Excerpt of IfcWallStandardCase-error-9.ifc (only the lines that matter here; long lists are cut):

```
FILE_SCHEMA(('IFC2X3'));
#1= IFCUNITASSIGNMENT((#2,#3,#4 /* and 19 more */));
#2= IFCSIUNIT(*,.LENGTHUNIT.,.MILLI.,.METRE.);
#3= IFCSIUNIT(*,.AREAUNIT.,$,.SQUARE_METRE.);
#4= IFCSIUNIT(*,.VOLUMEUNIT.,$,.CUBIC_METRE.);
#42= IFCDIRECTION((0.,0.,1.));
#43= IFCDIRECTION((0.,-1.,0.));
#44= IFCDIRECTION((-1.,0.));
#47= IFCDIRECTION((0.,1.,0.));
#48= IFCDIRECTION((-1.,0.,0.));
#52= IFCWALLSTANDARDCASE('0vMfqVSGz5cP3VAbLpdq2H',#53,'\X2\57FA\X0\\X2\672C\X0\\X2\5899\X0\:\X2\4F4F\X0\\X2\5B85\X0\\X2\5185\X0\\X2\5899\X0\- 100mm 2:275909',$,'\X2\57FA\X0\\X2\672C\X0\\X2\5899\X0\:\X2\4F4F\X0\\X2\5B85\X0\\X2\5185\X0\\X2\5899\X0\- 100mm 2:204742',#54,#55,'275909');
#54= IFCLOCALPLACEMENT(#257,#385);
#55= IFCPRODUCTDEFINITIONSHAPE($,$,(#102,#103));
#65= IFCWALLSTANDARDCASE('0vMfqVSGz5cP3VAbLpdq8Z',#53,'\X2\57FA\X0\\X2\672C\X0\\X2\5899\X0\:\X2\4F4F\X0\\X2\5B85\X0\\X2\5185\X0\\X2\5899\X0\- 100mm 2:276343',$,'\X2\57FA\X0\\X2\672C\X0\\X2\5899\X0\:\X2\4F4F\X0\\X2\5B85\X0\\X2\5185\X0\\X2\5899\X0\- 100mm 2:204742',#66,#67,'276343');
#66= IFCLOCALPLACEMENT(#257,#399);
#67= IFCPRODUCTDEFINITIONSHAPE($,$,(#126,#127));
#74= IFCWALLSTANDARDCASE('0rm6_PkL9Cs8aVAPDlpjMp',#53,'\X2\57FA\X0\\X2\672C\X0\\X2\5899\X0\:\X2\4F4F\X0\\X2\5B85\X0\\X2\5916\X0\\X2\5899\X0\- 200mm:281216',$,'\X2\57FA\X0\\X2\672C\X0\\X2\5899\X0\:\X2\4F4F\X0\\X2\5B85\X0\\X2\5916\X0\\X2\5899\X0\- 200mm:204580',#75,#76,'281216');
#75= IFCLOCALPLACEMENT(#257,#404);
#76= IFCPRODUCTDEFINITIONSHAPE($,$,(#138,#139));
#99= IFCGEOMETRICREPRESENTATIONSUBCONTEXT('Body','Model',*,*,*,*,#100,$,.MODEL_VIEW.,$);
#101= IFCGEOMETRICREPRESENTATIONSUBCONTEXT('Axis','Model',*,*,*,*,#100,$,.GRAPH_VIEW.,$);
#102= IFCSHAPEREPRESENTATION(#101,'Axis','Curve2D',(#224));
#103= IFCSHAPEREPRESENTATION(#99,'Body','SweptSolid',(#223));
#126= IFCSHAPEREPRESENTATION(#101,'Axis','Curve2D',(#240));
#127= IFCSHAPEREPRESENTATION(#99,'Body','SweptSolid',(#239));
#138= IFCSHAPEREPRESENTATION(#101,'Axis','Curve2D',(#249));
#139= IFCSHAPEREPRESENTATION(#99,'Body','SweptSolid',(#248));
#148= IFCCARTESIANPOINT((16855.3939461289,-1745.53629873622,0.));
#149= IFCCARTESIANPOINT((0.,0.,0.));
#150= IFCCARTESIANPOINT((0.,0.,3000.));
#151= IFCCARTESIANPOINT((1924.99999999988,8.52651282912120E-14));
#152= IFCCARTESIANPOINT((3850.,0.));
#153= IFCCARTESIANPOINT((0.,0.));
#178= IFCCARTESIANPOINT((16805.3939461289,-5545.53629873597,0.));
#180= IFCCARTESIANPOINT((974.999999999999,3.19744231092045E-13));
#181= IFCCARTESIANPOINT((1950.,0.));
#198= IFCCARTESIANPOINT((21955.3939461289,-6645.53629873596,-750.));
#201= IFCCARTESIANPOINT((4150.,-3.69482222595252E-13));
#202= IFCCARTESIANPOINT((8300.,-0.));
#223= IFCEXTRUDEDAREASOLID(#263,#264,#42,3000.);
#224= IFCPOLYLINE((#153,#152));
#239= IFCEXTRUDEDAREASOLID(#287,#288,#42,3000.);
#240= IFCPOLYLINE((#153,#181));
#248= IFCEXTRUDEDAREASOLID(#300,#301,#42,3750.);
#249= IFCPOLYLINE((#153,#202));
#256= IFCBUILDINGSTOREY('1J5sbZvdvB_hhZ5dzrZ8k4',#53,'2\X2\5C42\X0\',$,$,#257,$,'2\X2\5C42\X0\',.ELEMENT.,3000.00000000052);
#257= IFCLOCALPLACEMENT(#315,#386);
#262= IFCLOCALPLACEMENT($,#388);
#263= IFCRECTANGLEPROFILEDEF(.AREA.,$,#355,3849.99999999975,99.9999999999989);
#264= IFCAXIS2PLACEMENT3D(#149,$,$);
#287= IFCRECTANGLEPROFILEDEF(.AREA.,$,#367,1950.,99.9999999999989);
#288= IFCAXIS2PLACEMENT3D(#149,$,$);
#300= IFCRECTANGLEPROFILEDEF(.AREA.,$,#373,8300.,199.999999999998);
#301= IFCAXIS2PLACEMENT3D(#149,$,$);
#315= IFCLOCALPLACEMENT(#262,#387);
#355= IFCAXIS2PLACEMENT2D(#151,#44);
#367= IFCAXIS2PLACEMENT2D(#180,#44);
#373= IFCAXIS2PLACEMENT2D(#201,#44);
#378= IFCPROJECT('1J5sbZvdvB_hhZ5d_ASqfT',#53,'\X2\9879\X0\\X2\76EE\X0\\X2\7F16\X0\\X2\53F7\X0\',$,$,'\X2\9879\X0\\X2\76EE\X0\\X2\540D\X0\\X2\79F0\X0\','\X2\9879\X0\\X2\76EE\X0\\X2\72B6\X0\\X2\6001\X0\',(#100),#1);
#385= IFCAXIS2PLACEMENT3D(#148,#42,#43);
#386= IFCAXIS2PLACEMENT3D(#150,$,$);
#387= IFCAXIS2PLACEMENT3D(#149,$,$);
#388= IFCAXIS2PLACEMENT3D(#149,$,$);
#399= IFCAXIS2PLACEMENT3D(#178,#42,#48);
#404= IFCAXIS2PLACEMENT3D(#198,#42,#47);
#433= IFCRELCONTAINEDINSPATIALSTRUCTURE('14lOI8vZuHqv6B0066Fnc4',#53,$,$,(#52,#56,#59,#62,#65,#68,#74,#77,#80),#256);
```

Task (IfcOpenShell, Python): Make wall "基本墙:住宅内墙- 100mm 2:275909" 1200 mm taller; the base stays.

```python
import ifcopenshell
import ifcopenshell.geom
import ifcopenshell.util.representation
import ifcopenshell.util.shape

model = ifcopenshell.open("IfcWallStandardCase-error-9.ifc")
settings = ifcopenshell.geom.settings()


def volume(element):
    """Net volume in cubic metres, openings subtracted."""
    shape = ifcopenshell.geom.create_shape(settings, element)
    return ifcopenshell.util.shape.get_volume(shape.geometry)


wall = model.by_guid("0vMfqVSGz5cP3VAbLpdq2H")
before = volume(wall)

body = ifcopenshell.util.representation.get_representation(wall, "Model", "Body")
solid = body.Items[0]
old_height = solid.Depth
solid.Depth += 1200.0
after = volume(wall)

print(f"height {old_height:g} -> {solid.Depth:g}, volume {before:.3f} -> {after:.3f} m3")

model.write("IfcWallStandardCase-error-9-out.ifc")
```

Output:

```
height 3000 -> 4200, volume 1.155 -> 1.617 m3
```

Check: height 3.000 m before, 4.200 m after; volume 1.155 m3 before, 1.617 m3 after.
